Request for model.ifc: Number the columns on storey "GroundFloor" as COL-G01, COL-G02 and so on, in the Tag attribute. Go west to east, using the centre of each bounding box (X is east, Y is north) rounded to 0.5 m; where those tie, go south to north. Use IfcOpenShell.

First a look at what the model holds.

```python
import ifcopenshell
import ifcopenshell.util.element
import ifcopenshell.util.placement

model = ifcopenshell.open("model.ifc")
print(model.schema)
storey = next(s for s in model.by_type("IfcBuildingStorey") if s.Name == "GroundFloor")
columns = [e for e in ifcopenshell.util.element.get_decomposition(storey) if e.is_a("IfcColumn")]
for e in sorted(columns, key=lambda e: e.id()):
    origin = ifcopenshell.util.placement.get_local_placement(e.ObjectPlacement)[:3, 3]
    print(e.id(), e.Tag, e.Name, origin.round(2) + 0.0, sep=" | ")
```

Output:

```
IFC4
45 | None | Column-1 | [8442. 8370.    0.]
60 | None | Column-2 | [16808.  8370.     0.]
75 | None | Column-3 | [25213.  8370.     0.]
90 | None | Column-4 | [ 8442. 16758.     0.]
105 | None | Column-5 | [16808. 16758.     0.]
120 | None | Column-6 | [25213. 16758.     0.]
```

```python
import ifcopenshell
import ifcopenshell.geom
import ifcopenshell.util.element
import ifcopenshell.util.shape

model = ifcopenshell.open("model.ifc")
settings = ifcopenshell.geom.settings()
settings.set("use-world-coords", True)


def centre(element):
    shape = ifcopenshell.geom.create_shape(settings, element)
    return ifcopenshell.util.shape.get_bbox_centroid(shape.geometry)


storey = next(s for s in model.by_type("IfcBuildingStorey") if s.Name == "GroundFloor")
columns = [e for e in ifcopenshell.util.element.get_decomposition(storey) if e.is_a("IfcColumn")]

# Insertion points can sit at a corner or the storey origin, so sort by the geometry (in metres).
centres = {e: centre(e) for e in columns}
columns.sort(key=lambda e: (round(centres[e][0] / 0.5), centres[e][1]))

for i, e in enumerate(columns, start=1):
    number = f"COL-G{i:02d}"
    e.Tag = number
    print(e.id(), number)

model.write("model_rev.ifc")
```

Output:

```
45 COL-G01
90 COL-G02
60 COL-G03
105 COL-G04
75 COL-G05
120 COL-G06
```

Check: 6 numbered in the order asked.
